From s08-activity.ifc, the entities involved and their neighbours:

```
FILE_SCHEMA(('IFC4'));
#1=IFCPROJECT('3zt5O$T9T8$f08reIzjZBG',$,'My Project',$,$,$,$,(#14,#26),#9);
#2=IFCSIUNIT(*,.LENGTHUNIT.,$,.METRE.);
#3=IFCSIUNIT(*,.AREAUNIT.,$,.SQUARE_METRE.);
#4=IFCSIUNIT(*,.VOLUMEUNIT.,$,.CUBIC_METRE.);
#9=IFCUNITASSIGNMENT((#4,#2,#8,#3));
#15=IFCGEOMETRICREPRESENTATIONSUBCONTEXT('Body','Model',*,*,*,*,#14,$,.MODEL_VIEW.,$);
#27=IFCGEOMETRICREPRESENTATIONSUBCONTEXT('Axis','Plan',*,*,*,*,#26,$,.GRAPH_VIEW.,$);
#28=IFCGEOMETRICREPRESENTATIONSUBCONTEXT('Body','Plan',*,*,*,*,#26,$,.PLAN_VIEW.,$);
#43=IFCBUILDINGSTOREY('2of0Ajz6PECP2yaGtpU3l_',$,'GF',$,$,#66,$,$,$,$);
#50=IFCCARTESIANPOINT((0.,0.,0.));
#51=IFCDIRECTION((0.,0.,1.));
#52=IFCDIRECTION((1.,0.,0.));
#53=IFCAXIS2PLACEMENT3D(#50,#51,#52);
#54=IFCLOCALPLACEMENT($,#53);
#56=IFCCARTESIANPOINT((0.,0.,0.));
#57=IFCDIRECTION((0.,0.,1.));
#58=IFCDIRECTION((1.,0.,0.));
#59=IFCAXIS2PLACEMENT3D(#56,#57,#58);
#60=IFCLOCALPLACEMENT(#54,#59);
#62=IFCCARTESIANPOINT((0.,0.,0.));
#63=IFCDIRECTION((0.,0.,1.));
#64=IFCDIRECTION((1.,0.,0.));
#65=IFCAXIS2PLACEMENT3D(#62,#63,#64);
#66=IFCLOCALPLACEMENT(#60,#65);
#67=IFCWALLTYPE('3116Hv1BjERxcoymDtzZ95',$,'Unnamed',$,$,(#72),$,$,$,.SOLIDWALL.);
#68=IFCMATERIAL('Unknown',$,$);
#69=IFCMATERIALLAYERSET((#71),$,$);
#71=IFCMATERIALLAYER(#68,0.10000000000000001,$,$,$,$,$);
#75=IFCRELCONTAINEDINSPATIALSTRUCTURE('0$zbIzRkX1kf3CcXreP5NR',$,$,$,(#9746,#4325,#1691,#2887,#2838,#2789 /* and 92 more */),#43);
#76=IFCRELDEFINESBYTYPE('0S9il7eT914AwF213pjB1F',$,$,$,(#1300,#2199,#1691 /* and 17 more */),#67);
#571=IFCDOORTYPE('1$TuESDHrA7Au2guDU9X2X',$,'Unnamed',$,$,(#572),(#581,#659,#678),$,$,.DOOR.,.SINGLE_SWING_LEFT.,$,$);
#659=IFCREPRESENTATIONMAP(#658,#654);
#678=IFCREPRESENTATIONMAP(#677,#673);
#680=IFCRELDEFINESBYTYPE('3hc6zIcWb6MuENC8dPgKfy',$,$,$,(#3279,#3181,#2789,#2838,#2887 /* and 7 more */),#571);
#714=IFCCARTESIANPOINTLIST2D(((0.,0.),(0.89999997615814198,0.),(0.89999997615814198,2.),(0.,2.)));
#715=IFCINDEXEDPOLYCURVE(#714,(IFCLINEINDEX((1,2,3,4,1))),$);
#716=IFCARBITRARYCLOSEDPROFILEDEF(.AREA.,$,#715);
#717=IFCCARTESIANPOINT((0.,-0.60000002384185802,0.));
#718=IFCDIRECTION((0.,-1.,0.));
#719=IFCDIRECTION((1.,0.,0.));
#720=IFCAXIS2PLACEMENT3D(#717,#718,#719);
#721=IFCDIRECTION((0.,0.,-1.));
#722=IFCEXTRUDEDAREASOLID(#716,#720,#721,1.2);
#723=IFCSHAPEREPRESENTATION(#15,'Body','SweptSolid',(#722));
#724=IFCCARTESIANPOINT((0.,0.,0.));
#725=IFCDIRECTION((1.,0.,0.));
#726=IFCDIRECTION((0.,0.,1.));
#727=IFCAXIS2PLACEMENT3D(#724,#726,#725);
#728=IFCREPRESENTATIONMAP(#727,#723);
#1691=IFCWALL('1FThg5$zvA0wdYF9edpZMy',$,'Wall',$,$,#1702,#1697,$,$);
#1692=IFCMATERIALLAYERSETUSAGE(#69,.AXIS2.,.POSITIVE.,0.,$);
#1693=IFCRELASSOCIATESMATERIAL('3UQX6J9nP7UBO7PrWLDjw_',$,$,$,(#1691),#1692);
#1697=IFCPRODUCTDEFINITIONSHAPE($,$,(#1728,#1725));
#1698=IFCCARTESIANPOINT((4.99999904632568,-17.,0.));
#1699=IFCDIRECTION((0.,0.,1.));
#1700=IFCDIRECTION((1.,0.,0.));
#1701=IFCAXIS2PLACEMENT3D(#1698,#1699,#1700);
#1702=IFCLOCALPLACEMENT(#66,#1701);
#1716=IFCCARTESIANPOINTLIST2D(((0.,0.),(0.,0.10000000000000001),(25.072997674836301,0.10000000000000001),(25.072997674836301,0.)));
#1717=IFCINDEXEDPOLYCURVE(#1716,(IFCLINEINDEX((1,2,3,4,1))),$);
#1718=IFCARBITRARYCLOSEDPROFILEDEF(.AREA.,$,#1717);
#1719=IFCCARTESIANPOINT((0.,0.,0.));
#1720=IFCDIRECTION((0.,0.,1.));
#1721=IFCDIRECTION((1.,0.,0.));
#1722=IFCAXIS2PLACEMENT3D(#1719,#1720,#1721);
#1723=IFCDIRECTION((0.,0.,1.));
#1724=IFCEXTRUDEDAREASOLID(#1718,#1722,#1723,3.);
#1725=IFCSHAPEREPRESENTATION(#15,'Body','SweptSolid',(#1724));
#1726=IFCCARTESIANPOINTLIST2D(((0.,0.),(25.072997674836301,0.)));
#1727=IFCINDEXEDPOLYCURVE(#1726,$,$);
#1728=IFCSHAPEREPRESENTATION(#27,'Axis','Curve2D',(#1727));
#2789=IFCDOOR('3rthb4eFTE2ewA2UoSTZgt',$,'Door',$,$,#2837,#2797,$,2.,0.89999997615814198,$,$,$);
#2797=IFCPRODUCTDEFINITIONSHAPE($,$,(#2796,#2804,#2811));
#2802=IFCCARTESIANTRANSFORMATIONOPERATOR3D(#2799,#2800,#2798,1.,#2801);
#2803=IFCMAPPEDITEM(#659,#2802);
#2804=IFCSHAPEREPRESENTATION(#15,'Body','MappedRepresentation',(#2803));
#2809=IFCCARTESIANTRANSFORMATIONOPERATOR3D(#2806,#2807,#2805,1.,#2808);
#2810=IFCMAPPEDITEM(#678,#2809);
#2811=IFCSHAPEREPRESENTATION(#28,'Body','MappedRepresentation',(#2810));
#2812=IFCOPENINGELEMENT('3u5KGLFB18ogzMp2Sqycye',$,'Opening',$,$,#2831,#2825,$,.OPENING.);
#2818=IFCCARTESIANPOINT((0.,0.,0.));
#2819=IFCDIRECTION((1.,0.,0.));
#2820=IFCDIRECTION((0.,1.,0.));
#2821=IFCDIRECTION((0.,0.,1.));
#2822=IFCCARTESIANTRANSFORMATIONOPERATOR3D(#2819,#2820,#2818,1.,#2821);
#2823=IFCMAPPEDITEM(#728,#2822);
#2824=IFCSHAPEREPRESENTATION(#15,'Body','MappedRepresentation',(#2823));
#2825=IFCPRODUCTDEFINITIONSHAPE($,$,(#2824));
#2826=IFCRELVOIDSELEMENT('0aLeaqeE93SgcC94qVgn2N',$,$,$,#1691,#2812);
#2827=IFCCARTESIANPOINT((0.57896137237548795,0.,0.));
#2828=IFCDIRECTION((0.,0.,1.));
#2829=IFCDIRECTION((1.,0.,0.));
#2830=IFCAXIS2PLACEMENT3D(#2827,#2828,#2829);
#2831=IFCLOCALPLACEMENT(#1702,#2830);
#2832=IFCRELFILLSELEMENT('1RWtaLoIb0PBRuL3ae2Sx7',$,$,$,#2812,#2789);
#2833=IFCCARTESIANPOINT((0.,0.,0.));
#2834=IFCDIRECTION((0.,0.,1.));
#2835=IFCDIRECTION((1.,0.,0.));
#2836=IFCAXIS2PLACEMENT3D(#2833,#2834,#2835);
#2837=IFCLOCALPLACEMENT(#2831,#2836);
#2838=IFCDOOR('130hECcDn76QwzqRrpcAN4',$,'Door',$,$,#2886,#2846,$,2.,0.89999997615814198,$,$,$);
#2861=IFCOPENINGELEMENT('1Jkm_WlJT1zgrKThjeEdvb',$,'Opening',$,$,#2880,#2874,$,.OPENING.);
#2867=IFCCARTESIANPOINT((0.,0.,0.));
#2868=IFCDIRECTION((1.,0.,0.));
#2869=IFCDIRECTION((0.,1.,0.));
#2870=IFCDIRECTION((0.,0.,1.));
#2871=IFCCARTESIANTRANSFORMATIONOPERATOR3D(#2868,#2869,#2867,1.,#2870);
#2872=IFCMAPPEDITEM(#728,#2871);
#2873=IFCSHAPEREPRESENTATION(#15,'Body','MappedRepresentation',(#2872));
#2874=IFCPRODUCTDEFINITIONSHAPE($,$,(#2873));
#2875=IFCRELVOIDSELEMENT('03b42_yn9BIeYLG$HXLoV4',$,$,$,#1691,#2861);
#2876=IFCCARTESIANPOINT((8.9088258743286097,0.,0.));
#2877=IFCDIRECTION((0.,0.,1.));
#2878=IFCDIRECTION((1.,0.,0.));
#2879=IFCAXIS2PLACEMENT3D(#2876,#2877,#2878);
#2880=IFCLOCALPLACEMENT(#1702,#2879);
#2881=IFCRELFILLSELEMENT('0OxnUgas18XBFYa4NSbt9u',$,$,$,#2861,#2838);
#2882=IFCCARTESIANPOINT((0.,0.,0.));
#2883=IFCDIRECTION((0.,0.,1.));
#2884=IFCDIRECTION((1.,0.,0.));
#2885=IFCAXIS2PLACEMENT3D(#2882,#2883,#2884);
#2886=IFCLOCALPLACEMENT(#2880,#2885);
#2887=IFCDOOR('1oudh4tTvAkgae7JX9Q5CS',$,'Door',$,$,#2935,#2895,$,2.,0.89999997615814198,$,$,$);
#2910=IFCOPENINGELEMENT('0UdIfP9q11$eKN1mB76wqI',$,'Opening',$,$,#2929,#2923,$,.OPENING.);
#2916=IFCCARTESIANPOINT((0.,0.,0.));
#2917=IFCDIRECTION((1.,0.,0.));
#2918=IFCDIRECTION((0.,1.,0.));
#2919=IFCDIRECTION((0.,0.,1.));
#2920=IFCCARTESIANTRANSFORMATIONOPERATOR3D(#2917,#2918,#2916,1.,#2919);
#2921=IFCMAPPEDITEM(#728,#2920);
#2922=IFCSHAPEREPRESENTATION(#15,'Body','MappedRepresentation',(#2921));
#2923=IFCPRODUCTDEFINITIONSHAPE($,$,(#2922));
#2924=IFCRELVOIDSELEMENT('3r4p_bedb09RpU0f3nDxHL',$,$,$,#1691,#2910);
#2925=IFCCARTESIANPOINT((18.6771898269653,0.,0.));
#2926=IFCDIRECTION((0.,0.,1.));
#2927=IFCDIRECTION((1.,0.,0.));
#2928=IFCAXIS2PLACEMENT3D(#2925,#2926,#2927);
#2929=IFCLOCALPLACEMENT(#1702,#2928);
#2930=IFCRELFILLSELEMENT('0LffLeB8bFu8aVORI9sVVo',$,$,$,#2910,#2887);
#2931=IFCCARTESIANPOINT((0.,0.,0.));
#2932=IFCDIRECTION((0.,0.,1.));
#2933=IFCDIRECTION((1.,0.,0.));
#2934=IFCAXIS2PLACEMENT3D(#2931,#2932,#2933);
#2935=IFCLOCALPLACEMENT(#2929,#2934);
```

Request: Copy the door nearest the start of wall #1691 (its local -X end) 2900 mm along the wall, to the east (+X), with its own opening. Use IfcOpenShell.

```python
import ifcopenshell
import ifcopenshell.api.feature
import ifcopenshell.api.geometry
import ifcopenshell.api.root
import ifcopenshell.geom
import ifcopenshell.util.element
import ifcopenshell.util.placement
import ifcopenshell.util.shape

model = ifcopenshell.open("s08-activity.ifc")
settings = ifcopenshell.geom.settings()


def volume(element):
    """Net volume in cubic metres, openings subtracted."""
    shape = ifcopenshell.geom.create_shape(settings, element)
    return ifcopenshell.util.shape.get_volume(shape.geometry)


door = model.by_guid("3rthb4eFTE2ewA2UoSTZgt")
opening = door.FillsVoids[0].RelatingOpeningElement
wall = opening.VoidsElements[0].RelatingBuildingElement
before = volume(wall)
shift = ifcopenshell.util.placement.get_local_placement(wall.ObjectPlacement)[:3, 0] * 2.9

# copy_class copies the void relationship, type, container and properties, but no geometry.
new_opening = ifcopenshell.api.root.copy_class(model, product=opening)
new_opening.Representation = ifcopenshell.util.element.copy_deep(
    model, opening.Representation, exclude=["IfcGeometricRepresentationContext", "IfcRepresentationMap"]
)
new_door = ifcopenshell.api.root.copy_class(model, product=door)
new_door.Representation = ifcopenshell.util.element.copy_deep(
    model, door.Representation, exclude=["IfcGeometricRepresentationContext", "IfcRepresentationMap"]
)
ifcopenshell.api.feature.add_filling(model, opening=new_opening, element=new_door)

for old, new in ((opening, new_opening), (door, new_door)):
    matrix = ifcopenshell.util.placement.get_local_placement(old.ObjectPlacement)
    matrix[:3, 3] += shift
    ifcopenshell.api.geometry.edit_object_placement(model, product=new, matrix=matrix, is_si=False)

after = volume(wall)

print(f"wall volume {before:.3f} -> {after:.3f} m3")

model.write("s08-activity-out.ifc")
```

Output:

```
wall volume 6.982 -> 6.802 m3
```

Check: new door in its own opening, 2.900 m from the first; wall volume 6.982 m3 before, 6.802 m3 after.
